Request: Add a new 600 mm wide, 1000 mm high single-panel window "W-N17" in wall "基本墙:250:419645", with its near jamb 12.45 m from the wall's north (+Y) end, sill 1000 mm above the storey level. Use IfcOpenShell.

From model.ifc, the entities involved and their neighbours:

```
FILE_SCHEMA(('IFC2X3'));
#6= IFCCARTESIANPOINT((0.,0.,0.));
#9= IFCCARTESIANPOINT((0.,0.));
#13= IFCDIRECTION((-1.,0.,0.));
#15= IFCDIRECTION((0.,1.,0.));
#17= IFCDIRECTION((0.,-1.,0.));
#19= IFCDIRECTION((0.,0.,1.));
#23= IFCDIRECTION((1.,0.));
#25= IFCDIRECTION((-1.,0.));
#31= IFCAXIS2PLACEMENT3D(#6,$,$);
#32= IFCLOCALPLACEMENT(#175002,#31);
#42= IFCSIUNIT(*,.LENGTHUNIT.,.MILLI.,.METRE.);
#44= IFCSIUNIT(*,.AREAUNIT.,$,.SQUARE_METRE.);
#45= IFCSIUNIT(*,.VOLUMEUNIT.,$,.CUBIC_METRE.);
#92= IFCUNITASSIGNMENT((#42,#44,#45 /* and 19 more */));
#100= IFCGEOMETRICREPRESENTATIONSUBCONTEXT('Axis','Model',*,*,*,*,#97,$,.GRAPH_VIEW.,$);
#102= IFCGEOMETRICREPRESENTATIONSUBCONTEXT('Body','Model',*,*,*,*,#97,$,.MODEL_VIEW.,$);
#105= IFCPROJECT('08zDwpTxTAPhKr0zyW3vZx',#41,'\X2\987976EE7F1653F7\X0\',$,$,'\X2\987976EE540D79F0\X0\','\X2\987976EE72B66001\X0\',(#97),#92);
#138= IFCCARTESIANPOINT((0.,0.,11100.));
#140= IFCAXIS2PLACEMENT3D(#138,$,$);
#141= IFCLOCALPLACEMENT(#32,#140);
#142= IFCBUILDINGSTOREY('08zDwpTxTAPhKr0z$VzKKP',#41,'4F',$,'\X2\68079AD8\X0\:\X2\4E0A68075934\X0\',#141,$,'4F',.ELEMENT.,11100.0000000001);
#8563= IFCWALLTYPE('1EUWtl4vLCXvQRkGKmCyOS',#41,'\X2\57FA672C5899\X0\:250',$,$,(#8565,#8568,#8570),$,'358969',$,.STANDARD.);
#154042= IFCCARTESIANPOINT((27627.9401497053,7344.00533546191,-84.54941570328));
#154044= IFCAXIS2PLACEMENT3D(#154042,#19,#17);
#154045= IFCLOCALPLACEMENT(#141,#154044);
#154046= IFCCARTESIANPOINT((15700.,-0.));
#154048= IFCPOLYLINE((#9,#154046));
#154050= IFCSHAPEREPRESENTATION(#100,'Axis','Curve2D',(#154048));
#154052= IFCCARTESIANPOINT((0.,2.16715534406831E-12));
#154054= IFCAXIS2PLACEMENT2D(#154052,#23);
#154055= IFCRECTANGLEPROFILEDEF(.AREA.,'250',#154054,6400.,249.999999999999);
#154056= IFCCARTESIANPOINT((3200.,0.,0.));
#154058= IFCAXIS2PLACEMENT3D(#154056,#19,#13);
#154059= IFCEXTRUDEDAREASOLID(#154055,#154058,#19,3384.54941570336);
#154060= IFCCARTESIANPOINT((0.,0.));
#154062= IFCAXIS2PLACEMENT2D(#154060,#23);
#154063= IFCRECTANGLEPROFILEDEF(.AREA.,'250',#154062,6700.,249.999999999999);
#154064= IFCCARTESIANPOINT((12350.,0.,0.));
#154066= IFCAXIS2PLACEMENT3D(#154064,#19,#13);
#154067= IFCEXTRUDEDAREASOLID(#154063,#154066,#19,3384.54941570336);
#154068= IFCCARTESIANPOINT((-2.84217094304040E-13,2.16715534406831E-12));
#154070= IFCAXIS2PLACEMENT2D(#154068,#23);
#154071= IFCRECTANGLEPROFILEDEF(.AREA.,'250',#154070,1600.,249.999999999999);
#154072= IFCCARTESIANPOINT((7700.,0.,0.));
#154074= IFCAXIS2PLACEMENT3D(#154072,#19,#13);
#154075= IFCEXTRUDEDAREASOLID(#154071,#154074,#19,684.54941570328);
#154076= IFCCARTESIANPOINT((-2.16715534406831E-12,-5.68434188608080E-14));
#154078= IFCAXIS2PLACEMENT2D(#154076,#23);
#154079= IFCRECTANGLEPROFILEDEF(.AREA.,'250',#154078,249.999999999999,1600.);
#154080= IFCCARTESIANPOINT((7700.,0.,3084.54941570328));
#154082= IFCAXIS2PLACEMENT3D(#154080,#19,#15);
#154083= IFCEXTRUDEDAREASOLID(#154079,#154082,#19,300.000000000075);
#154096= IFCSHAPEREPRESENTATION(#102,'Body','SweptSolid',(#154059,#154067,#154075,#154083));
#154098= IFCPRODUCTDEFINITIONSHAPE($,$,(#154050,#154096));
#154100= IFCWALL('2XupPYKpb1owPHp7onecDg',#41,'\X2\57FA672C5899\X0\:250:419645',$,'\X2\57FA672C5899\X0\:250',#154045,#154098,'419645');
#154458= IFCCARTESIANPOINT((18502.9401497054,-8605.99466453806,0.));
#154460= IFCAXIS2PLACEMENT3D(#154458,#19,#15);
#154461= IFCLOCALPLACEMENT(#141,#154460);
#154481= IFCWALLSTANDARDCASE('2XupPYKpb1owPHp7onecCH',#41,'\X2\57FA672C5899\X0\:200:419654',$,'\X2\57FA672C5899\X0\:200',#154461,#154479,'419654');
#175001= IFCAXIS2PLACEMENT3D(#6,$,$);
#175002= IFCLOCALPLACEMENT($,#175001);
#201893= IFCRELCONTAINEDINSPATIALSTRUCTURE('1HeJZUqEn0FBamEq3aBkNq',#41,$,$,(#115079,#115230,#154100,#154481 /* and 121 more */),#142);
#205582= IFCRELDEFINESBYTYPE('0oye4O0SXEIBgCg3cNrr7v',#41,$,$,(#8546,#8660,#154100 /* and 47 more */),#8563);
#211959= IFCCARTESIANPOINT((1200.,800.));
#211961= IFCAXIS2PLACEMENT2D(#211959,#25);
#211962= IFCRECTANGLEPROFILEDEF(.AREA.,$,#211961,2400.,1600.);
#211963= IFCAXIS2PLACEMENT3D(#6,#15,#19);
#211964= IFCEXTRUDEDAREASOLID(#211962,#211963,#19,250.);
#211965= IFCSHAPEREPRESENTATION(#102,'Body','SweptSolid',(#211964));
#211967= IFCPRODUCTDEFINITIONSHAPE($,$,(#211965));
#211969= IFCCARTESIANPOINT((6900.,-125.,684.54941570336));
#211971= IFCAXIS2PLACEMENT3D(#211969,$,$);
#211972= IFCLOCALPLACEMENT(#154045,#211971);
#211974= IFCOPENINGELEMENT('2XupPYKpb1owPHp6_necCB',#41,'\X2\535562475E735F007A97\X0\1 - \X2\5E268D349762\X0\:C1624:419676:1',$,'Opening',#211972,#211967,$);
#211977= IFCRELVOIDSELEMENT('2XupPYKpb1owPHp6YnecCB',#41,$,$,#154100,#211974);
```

```python
import numpy as np
import ifcopenshell
import ifcopenshell.api.feature
import ifcopenshell.api.geometry
import ifcopenshell.api.root
import ifcopenshell.api.spatial
import ifcopenshell.api.type
import ifcopenshell.geom
import ifcopenshell.util.element
import ifcopenshell.util.placement
import ifcopenshell.util.representation
import ifcopenshell.util.shape
import ifcopenshell.util.unit

model = ifcopenshell.open("model.ifc")
unit_scale = ifcopenshell.util.unit.calculate_unit_scale(model)
settings = ifcopenshell.geom.settings()


def volume(element):
    """Net volume in cubic metres, openings subtracted."""
    shape = ifcopenshell.geom.create_shape(settings, element)
    return ifcopenshell.util.shape.get_volume(shape.geometry)


wall = model.by_guid("2XupPYKpb1owPHp7onecDg")
storey = ifcopenshell.util.element.get_container(wall, ifc_class="IfcBuildingStorey")
context = ifcopenshell.util.representation.get_context(model, "Model", "Body", "MODEL_VIEW")
before = volume(wall)

width, height, from_end, sill = 0.6, 1, 12.45, 1  # metres

# The wall runs along its own X axis, and the end named is its -X end.
wall_shape = ifcopenshell.geom.create_shape(settings, wall)
x, y, z = ifcopenshell.util.shape.get_vertices(wall_shape.geometry).T
start = x.min() + from_end
face, thickness = float(y.min()), float(y.max() - y.min())
wall_matrix = ifcopenshell.util.placement.get_local_placement(wall.ObjectPlacement)
level = ifcopenshell.util.placement.get_local_placement(storey.ObjectPlacement)[2, 3]


def in_wall(x, y):
    """Placement at x, y metres in the wall's axes, at sill height."""
    matrix = wall_matrix.copy()
    matrix[:, 3] = wall_matrix @ np.array([x / unit_scale, y / unit_scale, 0.0, 1.0])
    matrix[2, 3] = level + sill / unit_scale
    return matrix


# Opening: a box that overshoots both wall faces by 50 mm.
opening = ifcopenshell.api.root.create_entity(model, ifc_class="IfcOpeningElement")
box = ifcopenshell.api.geometry.add_wall_representation(
    model, context=context, length=width, height=height, thickness=thickness + 0.1
)
ifcopenshell.api.geometry.assign_representation(model, product=opening, representation=box)
ifcopenshell.api.geometry.edit_object_placement(model, product=opening, matrix=in_wall(start, face - 0.05), is_si=False)
ifcopenshell.api.feature.add_feature(model, feature=opening, element=wall)

window = ifcopenshell.api.root.create_entity(model, ifc_class="IfcWindow", name="W-N17")
window.OverallWidth, window.OverallHeight = width / unit_scale, height / unit_scale
body = ifcopenshell.api.geometry.add_window_representation(
    model,
    context=context,
    overall_width=window.OverallWidth,
    overall_height=window.OverallHeight,
    partition_type="SINGLE_PANEL",
)
ifcopenshell.api.geometry.assign_representation(model, product=window, representation=body)
ifcopenshell.api.spatial.assign_container(model, products=[window], relating_structure=storey)
fills = ifcopenshell.api.feature.add_filling(model, opening=opening, element=window)
fills.OwnerHistory = window.OwnerHistory  # required in IFC2X3

# IFC2X3 keeps the operation on the window style.
style = ifcopenshell.api.root.create_entity(model, ifc_class="IfcWindowStyle", name="W-N17")
style.OperationType, style.ConstructionType = "SINGLE_PANEL", "NOTDEFINED"
style.ParameterTakesPrecedence = style.Sizeable = False
ifcopenshell.api.type.assign_type(model, related_objects=[window], relating_type=style)

# Centre the window in the wall's thickness.
ifcopenshell.api.geometry.edit_object_placement(model, product=window, matrix=in_wall(start, face), is_si=False)
window_shape = ifcopenshell.geom.create_shape(settings, window)
depth = ifcopenshell.util.shape.get_vertices(window_shape.geometry)[:, 1]
offset = face + thickness / 2 - (depth.min() + depth.max()) / 2
ifcopenshell.api.geometry.edit_object_placement(model, product=window, matrix=in_wall(start, offset), is_si=False)

after = volume(wall)

print(f"wall volume {before:.3f} -> {after:.3f} m3")

model.write("model_updated.ifc")
```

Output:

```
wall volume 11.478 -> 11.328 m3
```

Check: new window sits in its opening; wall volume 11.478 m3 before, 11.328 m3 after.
